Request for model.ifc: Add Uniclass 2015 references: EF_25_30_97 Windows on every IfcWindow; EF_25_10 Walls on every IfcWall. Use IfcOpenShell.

First a look at what the model holds.

```python
import ifcopenshell

model = ifcopenshell.open("model.ifc")
print(model.schema)
print("classifications:", [c.Name for c in model.by_type("IfcClassification")])
for ifc_class in ("IfcDoor", "IfcRoof", "IfcStair", "IfcWall", "IfcWindow"):
    print(ifc_class, len(model.by_type(ifc_class)))
```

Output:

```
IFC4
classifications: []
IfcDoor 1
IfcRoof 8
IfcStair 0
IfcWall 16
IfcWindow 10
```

```python
import ifcopenshell
import ifcopenshell.api.classification

model = ifcopenshell.open("model.ifc")

system = ifcopenshell.api.classification.add_classification(model, classification="Uniclass 2015")

codes = {
    "IfcWindow": ("EF_25_30_97", "Windows"),
    "IfcWall": ("EF_25_10", "Walls"),
}
for ifc_class, (code, name) in codes.items():
    products = model.by_type(ifc_class)
    ifcopenshell.api.classification.add_reference(
        model, products=products, classification=system, identification=code, name=name
    )
    print(code, len(products))

model.write("model_rev.ifc")
```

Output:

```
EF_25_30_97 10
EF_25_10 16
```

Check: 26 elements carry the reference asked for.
